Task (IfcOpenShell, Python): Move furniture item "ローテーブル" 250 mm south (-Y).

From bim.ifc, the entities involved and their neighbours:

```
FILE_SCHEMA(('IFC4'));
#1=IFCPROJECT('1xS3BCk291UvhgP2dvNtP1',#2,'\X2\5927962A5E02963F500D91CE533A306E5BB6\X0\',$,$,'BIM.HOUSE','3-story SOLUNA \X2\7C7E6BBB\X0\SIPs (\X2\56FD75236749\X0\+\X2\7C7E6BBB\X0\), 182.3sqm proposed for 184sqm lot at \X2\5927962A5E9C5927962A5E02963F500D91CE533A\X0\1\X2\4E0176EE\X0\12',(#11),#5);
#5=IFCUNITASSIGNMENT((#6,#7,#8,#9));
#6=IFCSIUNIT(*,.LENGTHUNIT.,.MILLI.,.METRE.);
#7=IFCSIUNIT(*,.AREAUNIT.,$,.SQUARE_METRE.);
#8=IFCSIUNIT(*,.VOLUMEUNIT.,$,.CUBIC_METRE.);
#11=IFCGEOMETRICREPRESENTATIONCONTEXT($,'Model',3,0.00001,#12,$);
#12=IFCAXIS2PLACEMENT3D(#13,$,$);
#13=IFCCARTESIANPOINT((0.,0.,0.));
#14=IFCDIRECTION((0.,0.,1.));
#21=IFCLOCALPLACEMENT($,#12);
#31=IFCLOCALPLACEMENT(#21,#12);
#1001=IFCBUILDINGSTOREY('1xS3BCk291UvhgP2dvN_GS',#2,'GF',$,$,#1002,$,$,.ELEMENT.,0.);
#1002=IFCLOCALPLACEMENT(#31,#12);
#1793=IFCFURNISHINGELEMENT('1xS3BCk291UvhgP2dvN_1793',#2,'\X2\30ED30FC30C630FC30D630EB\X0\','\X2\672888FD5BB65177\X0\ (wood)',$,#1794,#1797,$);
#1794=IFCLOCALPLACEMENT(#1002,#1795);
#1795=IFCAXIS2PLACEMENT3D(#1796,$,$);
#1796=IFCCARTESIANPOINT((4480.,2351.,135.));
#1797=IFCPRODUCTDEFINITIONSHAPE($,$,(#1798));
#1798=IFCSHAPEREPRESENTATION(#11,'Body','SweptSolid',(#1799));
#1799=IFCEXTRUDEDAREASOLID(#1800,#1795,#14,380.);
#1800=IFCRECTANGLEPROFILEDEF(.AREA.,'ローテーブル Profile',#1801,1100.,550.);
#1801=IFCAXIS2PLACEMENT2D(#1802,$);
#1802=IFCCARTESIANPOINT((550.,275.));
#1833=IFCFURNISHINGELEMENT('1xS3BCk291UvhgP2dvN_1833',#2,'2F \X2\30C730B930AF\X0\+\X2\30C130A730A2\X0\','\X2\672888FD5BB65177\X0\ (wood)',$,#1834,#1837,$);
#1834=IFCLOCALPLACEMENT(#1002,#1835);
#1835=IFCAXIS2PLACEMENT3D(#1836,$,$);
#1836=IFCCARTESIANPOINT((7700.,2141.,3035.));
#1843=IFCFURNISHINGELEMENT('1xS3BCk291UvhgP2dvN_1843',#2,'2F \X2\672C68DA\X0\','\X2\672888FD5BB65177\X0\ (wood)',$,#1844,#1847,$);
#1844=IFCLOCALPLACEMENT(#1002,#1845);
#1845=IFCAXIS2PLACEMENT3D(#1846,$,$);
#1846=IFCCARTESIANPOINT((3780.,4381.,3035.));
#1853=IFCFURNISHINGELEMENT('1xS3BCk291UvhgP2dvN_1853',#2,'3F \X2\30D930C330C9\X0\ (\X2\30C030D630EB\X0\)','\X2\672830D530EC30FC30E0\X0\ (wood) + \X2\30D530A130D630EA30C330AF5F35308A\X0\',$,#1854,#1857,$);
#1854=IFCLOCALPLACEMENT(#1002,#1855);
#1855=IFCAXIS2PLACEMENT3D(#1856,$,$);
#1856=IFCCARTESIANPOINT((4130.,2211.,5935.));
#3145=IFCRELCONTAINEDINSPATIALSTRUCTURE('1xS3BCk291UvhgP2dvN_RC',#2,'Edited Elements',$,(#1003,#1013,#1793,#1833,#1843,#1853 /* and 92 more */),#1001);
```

```python
import ifcopenshell
import ifcopenshell.api.geometry
import ifcopenshell.util.placement

model = ifcopenshell.open("bim.ifc")

item = model.by_guid("1xS3BCk291UvhgP2dvN_1793")
matrix = ifcopenshell.util.placement.get_local_placement(item.ObjectPlacement)
matrix[1, 3] -= 250.0
ifcopenshell.api.geometry.edit_object_placement(model, product=item, matrix=matrix, is_si=False)

print(ifcopenshell.util.placement.get_local_placement(item.ObjectPlacement).round(3) + 0.0)

model.write("bim-out.ifc")
```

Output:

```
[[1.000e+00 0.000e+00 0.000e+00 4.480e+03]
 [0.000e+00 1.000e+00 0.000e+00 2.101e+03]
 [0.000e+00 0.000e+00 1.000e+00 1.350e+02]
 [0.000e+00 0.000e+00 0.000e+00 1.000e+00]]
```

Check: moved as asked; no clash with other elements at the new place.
